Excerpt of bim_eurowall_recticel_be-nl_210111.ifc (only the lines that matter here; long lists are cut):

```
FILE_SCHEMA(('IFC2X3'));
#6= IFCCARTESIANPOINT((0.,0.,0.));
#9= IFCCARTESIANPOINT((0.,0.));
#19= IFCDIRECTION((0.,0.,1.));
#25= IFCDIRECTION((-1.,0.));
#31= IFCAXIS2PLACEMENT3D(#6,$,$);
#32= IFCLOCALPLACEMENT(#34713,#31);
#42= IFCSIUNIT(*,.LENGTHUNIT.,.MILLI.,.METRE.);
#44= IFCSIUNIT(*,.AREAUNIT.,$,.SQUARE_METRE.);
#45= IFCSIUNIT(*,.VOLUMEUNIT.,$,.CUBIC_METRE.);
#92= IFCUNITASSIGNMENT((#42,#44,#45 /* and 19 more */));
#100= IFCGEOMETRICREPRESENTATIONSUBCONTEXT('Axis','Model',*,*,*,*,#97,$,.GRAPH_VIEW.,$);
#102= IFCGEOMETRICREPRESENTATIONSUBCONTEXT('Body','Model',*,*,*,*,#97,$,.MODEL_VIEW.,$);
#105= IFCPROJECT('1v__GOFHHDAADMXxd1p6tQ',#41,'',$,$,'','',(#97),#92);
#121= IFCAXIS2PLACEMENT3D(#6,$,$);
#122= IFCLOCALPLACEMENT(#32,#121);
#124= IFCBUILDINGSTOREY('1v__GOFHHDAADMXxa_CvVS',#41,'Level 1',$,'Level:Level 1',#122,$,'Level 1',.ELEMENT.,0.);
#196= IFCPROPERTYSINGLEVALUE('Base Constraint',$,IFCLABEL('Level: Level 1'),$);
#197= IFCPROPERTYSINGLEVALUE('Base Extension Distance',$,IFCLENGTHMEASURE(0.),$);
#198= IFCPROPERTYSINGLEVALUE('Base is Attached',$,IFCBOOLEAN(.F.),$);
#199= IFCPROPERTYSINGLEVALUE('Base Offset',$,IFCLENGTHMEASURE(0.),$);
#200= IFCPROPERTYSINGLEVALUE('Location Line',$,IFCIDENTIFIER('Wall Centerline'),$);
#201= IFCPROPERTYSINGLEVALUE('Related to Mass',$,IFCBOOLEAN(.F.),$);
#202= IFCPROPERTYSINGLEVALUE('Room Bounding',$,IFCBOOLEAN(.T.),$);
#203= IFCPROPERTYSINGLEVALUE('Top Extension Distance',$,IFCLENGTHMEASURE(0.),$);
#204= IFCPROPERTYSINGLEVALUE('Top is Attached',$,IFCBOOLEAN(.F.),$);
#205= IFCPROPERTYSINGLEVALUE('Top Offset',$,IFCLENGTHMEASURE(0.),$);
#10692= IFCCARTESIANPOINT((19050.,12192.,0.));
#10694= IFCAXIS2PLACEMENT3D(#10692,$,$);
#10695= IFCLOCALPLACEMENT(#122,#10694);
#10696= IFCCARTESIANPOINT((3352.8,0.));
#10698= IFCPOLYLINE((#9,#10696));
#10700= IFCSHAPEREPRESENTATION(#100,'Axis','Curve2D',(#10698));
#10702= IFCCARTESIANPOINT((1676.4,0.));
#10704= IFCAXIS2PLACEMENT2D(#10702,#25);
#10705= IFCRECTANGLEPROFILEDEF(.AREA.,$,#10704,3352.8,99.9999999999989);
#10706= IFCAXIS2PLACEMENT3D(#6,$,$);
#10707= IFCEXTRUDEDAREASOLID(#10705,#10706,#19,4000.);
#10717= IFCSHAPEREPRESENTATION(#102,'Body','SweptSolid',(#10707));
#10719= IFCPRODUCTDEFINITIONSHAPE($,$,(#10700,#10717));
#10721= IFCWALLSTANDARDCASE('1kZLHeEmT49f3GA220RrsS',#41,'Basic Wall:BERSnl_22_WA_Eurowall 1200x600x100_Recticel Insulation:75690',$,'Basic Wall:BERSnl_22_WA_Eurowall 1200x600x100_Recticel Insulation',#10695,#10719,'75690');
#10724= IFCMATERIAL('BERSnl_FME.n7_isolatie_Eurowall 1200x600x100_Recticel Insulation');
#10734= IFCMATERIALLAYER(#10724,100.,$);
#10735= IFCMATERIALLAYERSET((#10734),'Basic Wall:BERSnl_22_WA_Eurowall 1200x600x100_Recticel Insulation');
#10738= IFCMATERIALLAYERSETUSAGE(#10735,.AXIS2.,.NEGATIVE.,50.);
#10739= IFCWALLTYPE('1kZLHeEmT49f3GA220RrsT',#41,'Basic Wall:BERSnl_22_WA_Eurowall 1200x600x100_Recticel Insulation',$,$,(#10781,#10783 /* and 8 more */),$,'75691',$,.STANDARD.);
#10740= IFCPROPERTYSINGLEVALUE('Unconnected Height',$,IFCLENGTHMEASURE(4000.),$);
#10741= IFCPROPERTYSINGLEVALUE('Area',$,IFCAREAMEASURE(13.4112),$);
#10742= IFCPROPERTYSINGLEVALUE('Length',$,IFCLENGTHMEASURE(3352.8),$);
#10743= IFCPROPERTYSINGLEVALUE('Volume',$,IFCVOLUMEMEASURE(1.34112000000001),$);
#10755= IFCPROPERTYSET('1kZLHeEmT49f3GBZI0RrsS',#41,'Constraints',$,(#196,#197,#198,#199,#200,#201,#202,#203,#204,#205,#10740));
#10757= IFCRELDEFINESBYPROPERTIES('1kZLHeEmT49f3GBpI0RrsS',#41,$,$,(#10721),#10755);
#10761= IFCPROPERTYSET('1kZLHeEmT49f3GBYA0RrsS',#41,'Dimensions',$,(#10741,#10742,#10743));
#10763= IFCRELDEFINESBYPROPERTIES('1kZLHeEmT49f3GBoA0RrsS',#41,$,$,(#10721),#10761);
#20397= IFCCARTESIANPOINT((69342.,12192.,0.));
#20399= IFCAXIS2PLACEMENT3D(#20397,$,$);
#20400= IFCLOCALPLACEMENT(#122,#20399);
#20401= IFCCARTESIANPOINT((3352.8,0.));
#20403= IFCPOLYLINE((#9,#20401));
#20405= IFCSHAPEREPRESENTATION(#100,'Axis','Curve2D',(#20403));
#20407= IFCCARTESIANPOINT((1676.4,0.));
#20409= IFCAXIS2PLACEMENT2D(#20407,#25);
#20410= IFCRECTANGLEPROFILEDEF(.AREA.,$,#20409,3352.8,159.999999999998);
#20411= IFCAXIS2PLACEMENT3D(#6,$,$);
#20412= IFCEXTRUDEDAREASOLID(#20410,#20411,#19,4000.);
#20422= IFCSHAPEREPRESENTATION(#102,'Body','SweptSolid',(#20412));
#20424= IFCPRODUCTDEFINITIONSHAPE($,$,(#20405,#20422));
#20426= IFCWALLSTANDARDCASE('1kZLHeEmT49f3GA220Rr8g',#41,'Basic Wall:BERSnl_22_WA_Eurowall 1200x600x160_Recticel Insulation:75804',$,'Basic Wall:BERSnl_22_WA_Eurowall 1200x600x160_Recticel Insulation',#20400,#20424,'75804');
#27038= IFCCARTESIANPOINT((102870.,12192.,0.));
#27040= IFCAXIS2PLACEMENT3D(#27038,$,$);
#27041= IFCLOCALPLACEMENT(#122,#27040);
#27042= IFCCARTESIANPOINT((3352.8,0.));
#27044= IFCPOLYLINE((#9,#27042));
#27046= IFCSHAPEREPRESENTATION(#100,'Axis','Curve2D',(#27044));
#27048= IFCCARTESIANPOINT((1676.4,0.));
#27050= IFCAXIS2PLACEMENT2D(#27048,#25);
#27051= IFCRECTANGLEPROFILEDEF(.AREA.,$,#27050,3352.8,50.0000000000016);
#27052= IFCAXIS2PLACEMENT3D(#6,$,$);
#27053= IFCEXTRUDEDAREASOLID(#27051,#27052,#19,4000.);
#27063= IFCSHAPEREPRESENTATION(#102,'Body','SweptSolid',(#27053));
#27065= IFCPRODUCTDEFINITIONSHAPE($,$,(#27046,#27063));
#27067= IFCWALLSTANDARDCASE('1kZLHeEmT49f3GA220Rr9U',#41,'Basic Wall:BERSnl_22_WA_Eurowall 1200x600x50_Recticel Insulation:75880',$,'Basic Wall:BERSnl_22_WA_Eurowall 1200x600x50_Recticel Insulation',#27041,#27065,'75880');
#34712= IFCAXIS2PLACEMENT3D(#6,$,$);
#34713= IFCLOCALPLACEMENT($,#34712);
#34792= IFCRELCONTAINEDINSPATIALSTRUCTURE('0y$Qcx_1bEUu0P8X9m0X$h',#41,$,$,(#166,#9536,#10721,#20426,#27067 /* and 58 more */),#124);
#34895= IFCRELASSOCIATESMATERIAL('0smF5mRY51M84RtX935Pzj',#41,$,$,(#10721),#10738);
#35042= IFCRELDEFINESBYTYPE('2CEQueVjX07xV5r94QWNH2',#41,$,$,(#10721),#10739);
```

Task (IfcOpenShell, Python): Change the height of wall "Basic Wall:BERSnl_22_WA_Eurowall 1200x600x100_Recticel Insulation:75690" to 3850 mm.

```python
import ifcopenshell
import ifcopenshell.api.pset
import ifcopenshell.geom
import ifcopenshell.util.element
import ifcopenshell.util.representation
import ifcopenshell.util.shape
import ifcopenshell.util.unit

model = ifcopenshell.open("bim_eurowall_recticel_be-nl_210111.ifc")
area_scale = ifcopenshell.util.unit.calculate_unit_scale(model, "AREAUNIT")
volume_scale = ifcopenshell.util.unit.calculate_unit_scale(model, "VOLUMEUNIT")
settings = ifcopenshell.geom.settings()


def volume(element):
    """Net volume in cubic metres, openings subtracted."""
    shape = ifcopenshell.geom.create_shape(settings, element)
    return ifcopenshell.util.shape.get_volume(shape.geometry)


wall = model.by_guid("1kZLHeEmT49f3GA220RrsS")
before = volume(wall)

body = ifcopenshell.util.representation.get_representation(wall, "Model", "Body")
solid = body.Items[0]
old_height = solid.Depth
solid.Depth = 3850.0
after = volume(wall)
thickness = 0.1  # wall thickness in metres

# Update the stored height, areas and volumes.
pset = model.by_id(ifcopenshell.util.element.get_pset(wall, "Constraints", should_inherit=False)["id"])
ifcopenshell.api.pset.edit_pset(model, pset=pset, properties={
    "Unconnected Height": model.create_entity("IfcLengthMeasure", solid.Depth),
})
pset = model.by_id(ifcopenshell.util.element.get_pset(wall, "Dimensions", should_inherit=False)["id"])
ifcopenshell.api.pset.edit_pset(model, pset=pset, properties={
    "Area": model.create_entity("IfcAreaMeasure", after / thickness / area_scale),
    "Volume": model.create_entity("IfcVolumeMeasure", after / volume_scale),
})

print(f"height {old_height:g} -> {solid.Depth:g}, volume {before:.3f} -> {after:.3f} m3")

model.write("bim_eurowall_recticel_be-nl_210111_v2.ifc")
```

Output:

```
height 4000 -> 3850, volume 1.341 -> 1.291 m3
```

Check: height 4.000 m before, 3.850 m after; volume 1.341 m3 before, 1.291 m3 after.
